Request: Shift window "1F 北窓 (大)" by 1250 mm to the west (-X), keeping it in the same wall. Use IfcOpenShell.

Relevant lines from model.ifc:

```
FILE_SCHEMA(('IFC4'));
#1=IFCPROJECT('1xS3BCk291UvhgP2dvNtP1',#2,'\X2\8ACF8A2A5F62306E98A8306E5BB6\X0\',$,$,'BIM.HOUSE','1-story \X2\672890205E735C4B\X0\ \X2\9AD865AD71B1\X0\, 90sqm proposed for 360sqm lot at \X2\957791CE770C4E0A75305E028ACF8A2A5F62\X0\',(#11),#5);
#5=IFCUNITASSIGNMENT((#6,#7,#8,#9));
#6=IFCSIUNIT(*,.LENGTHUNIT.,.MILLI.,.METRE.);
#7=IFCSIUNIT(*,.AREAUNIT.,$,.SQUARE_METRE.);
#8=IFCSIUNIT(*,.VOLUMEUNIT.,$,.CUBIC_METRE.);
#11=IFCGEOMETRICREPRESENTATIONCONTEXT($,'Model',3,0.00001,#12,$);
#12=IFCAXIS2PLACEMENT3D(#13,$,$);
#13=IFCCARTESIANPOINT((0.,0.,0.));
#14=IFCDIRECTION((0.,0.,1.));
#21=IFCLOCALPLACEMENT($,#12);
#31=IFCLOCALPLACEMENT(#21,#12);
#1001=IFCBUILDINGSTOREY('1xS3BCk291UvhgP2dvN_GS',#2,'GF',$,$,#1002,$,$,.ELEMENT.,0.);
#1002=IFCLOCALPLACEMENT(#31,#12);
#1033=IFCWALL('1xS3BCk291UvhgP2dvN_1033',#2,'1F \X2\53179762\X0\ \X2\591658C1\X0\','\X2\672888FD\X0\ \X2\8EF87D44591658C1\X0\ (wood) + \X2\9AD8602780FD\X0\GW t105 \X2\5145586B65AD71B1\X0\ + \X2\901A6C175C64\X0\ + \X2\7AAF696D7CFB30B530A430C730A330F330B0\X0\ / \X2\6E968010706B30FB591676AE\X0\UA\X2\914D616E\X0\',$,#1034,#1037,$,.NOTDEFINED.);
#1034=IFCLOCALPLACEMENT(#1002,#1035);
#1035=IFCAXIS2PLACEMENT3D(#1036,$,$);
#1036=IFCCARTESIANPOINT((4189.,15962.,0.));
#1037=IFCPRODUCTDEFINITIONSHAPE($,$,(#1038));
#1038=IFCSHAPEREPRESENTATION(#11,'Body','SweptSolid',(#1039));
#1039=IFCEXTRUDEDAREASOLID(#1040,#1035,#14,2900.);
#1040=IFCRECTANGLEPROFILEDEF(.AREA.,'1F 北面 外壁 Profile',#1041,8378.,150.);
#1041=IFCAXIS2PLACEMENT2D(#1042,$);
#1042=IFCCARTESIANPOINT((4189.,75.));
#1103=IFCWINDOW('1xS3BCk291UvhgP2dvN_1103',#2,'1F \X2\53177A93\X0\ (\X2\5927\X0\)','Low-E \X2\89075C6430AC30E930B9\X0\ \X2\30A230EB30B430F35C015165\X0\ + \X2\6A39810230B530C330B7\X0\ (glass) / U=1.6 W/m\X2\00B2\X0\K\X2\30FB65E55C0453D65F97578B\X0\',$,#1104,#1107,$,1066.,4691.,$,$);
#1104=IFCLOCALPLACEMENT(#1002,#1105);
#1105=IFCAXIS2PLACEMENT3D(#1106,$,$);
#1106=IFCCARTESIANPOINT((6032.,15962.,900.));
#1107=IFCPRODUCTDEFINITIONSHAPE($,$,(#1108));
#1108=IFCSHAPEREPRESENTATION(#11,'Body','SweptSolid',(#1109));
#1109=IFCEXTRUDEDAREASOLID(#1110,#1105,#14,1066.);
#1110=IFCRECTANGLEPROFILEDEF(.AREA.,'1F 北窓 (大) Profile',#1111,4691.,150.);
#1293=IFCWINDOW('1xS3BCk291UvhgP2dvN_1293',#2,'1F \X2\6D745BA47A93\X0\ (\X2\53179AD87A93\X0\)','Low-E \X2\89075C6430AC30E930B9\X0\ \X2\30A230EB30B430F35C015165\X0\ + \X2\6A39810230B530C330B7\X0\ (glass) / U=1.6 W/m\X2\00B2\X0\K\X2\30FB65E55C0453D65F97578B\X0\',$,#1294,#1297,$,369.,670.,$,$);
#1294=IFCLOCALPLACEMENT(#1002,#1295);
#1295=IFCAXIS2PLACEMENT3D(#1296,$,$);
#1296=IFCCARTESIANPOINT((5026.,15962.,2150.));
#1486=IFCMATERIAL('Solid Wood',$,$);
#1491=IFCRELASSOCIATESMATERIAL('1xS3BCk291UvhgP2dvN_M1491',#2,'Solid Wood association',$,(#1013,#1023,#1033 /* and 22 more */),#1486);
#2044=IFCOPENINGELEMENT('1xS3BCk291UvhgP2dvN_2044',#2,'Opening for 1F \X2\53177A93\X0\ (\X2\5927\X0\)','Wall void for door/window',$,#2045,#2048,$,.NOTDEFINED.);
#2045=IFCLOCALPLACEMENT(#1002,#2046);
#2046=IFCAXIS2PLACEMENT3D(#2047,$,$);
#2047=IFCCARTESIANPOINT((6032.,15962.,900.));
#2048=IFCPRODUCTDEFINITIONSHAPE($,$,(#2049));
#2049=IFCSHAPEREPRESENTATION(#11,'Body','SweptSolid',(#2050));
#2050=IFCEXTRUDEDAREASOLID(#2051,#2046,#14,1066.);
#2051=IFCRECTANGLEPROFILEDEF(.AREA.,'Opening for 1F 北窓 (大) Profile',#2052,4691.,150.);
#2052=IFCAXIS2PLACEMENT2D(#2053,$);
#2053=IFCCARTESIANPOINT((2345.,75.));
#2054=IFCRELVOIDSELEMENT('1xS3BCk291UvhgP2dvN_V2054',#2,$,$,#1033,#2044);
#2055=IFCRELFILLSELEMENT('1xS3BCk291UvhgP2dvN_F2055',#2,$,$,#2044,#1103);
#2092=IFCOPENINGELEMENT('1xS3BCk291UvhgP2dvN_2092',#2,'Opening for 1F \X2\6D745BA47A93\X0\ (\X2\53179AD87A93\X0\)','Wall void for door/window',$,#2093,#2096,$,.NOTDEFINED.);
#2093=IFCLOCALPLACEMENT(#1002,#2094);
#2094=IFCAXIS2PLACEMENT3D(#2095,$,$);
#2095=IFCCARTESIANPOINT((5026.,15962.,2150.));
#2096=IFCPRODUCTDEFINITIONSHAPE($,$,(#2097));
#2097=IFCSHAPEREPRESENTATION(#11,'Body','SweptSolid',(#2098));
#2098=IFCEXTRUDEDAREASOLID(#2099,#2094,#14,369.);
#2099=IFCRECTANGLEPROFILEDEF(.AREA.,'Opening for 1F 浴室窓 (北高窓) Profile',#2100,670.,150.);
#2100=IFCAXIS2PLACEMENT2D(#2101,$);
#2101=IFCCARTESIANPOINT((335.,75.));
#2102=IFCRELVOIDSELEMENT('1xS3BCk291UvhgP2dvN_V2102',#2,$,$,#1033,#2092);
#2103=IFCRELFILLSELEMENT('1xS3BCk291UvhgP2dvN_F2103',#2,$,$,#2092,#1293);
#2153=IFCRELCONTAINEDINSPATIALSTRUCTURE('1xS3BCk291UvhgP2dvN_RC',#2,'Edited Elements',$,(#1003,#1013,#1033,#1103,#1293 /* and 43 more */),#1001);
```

```python
import ifcopenshell
import ifcopenshell.api.geometry
import ifcopenshell.util.placement

model = ifcopenshell.open("model.ifc")

window = model.by_guid("1xS3BCk291UvhgP2dvN_1103")
opening = window.FillsVoids[0].RelatingOpeningElement
wall = opening.VoidsElements[0].RelatingBuildingElement

wall_matrix = ifcopenshell.util.placement.get_local_placement(wall.ObjectPlacement)
shift = wall_matrix[:3, 0] * -1250.0
before = ifcopenshell.util.placement.get_local_placement(window.ObjectPlacement)[:3, 3].copy()

# The window is not placed relative to its opening, so move both.
for product in (opening, window):
    matrix = ifcopenshell.util.placement.get_local_placement(product.ObjectPlacement)
    matrix[:3, 3] += shift
    ifcopenshell.api.geometry.edit_object_placement(model, product=product, matrix=matrix, is_si=False)

after = ifcopenshell.util.placement.get_local_placement(window.ObjectPlacement)[:3, 3]
print("window moved by", (after - before).round(3) + 0.0)

model.write("model_rev.ifc")
```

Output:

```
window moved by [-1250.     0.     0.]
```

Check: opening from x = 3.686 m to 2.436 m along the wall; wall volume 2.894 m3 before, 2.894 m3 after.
